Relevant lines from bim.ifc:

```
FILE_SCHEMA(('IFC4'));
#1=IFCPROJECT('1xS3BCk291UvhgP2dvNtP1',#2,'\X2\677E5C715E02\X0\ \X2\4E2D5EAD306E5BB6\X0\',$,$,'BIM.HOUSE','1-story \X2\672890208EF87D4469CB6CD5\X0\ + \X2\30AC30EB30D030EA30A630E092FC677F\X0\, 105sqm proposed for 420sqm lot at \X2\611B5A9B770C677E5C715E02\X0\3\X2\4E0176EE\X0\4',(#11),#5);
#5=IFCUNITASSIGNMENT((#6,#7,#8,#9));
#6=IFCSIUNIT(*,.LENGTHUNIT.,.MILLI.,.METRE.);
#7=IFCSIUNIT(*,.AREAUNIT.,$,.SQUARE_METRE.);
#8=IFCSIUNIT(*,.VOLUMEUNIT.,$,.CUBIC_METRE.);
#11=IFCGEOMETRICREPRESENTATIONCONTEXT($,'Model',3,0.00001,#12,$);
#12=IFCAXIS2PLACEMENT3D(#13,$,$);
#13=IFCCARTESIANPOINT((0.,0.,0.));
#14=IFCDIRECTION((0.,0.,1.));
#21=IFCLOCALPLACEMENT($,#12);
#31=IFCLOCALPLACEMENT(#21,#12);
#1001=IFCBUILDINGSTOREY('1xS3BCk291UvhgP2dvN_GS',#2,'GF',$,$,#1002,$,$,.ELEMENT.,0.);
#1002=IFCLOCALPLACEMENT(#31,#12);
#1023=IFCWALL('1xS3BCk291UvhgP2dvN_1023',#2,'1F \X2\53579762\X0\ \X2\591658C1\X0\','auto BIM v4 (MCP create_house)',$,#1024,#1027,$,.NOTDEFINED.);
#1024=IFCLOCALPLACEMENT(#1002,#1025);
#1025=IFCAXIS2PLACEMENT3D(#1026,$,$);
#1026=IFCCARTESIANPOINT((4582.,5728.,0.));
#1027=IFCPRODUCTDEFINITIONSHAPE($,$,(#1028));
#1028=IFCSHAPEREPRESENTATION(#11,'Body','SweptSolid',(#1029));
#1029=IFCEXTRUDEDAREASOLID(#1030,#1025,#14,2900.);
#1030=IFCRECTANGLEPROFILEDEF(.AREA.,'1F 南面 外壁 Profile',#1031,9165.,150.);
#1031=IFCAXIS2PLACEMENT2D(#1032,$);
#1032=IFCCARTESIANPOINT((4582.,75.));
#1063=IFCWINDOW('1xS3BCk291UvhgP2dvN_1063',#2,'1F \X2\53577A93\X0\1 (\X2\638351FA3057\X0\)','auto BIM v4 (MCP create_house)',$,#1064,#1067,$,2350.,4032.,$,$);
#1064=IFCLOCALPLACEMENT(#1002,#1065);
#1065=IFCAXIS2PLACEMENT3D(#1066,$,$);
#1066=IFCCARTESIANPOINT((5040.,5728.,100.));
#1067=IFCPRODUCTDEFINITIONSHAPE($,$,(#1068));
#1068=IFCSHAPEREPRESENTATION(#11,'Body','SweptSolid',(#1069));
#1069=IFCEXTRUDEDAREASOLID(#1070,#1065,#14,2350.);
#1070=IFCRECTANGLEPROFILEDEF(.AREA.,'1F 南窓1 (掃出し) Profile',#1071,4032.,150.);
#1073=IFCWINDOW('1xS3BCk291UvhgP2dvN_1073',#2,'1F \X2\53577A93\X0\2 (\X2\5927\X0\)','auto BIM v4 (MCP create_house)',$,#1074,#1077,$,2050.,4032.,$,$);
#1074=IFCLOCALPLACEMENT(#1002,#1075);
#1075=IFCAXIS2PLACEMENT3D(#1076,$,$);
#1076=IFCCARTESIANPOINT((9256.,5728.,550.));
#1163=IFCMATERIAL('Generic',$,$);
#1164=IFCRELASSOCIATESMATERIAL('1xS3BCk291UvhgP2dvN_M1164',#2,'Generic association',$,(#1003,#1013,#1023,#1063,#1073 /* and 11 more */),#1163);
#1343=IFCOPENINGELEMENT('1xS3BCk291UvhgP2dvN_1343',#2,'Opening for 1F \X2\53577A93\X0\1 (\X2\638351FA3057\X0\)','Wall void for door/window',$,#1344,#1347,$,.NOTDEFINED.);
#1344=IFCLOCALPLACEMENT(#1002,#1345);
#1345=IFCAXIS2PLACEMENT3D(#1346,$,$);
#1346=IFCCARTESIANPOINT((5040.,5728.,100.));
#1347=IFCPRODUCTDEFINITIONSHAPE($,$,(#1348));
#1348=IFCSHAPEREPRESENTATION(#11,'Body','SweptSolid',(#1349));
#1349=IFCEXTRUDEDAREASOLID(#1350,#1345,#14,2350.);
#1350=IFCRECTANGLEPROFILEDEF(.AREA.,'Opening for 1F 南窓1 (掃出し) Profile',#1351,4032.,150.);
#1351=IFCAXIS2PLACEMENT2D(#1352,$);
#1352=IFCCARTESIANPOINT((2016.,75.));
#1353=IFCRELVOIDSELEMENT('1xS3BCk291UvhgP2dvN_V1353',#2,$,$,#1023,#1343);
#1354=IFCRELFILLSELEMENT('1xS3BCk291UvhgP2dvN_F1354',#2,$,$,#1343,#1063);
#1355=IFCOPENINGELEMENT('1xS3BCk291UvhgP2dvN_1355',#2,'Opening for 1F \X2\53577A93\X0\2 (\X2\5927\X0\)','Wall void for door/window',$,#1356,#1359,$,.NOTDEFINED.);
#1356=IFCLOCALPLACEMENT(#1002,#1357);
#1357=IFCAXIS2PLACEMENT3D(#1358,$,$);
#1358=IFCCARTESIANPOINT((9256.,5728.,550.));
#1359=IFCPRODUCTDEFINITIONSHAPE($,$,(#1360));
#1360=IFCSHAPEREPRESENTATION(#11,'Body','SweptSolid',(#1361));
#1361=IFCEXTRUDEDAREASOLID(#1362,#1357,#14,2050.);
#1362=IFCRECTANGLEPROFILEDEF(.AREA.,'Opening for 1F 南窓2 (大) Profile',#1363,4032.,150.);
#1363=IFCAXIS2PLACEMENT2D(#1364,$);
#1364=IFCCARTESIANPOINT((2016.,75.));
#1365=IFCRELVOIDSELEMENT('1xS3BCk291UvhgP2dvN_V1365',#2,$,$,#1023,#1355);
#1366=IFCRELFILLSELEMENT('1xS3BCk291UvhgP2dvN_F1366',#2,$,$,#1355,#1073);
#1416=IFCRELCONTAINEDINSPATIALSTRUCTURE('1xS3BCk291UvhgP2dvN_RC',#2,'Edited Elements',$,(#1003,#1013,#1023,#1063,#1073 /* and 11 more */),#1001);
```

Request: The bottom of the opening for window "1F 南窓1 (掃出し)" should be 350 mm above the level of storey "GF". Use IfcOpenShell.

```python
import numpy as np
import ifcopenshell
import ifcopenshell.api.geometry
import ifcopenshell.geom
import ifcopenshell.util.element
import ifcopenshell.util.placement
import ifcopenshell.util.shape
import ifcopenshell.util.unit

model = ifcopenshell.open("bim.ifc")
unit_scale = ifcopenshell.util.unit.calculate_unit_scale(model)

window = model.by_guid("1xS3BCk291UvhgP2dvN_1063")
opening = window.FillsVoids[0].RelatingOpeningElement
storey = ifcopenshell.util.element.get_container(window, ifc_class="IfcBuildingStorey")
level = ifcopenshell.util.placement.get_local_placement(storey.ObjectPlacement)[2, 3]

# The opening's origin need not be at the sill, so measure its lowest point.
shape = ifcopenshell.geom.create_shape(ifcopenshell.geom.settings(), opening)
bottom = ifcopenshell.util.shape.get_shape_bottom_elevation(shape, shape.geometry) / unit_scale
dz = level + 0.35 / unit_scale - bottom

shift = np.array([0.0, 0.0, dz])
# The window is not placed relative to its opening, so move both.
for product in (opening, window):
    matrix = ifcopenshell.util.placement.get_local_placement(product.ObjectPlacement)
    matrix[:3, 3] += shift
    ifcopenshell.api.geometry.edit_object_placement(model, product=product, matrix=matrix, is_si=False)

print(f"moved by {dz * unit_scale:+.3f} m")

model.write("bim_rev.ifc")
```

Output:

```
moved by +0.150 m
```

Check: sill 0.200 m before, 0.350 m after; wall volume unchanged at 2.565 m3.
